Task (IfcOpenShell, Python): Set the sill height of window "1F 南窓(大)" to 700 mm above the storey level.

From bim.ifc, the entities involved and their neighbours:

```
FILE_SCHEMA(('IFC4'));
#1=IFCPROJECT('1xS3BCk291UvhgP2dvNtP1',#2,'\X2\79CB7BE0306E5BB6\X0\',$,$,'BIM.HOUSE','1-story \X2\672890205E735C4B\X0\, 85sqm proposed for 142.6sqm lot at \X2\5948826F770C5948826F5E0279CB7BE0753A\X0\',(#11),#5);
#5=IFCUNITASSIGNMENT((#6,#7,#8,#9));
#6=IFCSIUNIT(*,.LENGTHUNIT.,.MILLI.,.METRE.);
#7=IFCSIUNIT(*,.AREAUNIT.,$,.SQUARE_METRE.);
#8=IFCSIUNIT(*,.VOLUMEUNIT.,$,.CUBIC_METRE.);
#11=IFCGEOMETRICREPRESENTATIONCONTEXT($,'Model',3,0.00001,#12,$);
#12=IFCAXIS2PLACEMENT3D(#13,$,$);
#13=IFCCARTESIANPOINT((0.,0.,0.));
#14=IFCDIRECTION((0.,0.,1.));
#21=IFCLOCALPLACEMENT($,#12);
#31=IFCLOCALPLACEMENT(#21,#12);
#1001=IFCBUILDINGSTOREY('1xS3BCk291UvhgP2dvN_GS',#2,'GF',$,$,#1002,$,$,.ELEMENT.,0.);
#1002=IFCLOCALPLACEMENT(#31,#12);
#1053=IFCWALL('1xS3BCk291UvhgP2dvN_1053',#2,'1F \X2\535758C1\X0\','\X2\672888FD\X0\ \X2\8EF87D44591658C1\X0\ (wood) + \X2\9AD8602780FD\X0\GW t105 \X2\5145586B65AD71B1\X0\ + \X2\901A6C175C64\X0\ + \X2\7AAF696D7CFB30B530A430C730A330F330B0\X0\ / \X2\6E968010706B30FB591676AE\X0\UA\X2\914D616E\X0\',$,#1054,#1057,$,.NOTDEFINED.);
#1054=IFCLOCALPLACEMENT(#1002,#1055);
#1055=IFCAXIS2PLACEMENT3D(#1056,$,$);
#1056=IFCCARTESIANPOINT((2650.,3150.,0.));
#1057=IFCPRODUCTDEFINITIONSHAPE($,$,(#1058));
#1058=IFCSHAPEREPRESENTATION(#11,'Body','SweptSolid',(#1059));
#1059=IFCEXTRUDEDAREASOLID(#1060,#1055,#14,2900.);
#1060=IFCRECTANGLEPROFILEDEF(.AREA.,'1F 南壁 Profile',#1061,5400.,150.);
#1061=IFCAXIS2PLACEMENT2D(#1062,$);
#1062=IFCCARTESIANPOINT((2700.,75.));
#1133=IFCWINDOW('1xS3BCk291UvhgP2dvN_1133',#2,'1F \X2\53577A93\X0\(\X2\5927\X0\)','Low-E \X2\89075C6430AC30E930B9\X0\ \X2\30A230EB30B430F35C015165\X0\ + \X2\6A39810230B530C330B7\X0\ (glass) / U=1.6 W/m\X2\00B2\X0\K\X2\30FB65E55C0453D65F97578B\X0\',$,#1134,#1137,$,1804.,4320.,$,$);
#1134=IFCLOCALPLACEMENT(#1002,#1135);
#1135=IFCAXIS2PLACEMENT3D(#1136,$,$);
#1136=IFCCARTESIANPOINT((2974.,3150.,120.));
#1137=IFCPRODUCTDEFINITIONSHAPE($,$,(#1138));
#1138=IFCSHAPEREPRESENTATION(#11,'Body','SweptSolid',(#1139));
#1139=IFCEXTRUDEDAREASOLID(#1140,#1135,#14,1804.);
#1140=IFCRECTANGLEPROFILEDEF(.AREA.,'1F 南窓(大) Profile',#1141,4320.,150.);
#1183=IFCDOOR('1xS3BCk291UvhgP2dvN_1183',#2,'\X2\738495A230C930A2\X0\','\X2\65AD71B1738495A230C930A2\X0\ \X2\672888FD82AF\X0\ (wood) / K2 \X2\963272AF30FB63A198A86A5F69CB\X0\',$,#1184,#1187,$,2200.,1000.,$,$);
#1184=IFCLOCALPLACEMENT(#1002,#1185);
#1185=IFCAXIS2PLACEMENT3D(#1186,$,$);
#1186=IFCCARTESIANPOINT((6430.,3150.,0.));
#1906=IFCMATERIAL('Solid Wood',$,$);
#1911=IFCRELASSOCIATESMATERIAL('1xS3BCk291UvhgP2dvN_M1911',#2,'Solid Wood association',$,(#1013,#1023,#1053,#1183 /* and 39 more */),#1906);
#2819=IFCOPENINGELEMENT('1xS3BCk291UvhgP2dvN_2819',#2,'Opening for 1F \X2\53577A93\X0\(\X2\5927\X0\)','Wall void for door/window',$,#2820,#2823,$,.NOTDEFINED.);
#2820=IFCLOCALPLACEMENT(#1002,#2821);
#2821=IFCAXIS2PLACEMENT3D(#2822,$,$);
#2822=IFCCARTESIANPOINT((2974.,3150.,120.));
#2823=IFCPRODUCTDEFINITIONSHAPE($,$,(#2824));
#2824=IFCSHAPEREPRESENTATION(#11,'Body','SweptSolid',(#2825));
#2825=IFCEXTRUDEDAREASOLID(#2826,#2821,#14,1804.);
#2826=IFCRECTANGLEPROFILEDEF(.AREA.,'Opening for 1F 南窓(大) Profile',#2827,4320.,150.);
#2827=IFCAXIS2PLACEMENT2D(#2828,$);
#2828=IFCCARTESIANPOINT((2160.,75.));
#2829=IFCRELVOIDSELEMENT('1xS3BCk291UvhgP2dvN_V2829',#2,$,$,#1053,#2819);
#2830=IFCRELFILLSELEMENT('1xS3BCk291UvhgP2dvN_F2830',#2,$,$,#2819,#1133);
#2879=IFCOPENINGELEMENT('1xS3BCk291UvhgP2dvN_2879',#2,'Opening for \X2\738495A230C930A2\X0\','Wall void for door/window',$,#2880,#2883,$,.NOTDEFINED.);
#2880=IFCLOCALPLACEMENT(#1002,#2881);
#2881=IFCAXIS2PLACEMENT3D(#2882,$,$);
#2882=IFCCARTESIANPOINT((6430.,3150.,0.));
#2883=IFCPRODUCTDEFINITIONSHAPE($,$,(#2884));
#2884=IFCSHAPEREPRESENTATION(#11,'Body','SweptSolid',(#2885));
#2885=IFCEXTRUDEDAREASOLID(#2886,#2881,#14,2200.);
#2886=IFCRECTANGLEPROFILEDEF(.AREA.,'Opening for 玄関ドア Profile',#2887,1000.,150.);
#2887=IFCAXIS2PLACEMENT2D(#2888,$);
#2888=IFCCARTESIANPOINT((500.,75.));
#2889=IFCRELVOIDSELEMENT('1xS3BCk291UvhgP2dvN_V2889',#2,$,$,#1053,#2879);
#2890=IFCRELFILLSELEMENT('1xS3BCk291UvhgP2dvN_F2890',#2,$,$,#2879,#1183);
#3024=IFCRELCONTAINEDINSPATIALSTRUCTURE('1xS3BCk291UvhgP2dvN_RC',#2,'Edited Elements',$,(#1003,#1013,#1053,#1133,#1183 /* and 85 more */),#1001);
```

```python
import numpy as np
import ifcopenshell
import ifcopenshell.api.geometry
import ifcopenshell.geom
import ifcopenshell.util.element
import ifcopenshell.util.placement
import ifcopenshell.util.shape
import ifcopenshell.util.unit

model = ifcopenshell.open("bim.ifc")
unit_scale = ifcopenshell.util.unit.calculate_unit_scale(model)

window = model.by_guid("1xS3BCk291UvhgP2dvN_1133")
opening = window.FillsVoids[0].RelatingOpeningElement
storey = ifcopenshell.util.element.get_container(window, ifc_class="IfcBuildingStorey")
level = ifcopenshell.util.placement.get_local_placement(storey.ObjectPlacement)[2, 3]

# The opening's origin need not be at the sill, so measure its lowest point.
shape = ifcopenshell.geom.create_shape(ifcopenshell.geom.settings(), opening)
bottom = ifcopenshell.util.shape.get_shape_bottom_elevation(shape, shape.geometry) / unit_scale
dz = level + 0.7 / unit_scale - bottom

shift = np.array([0.0, 0.0, dz])
# The window is not placed relative to its opening, so move both.
for product in (opening, window):
    matrix = ifcopenshell.util.placement.get_local_placement(product.ObjectPlacement)
    matrix[:3, 3] += shift
    ifcopenshell.api.geometry.edit_object_placement(model, product=product, matrix=matrix, is_si=False)

print(f"moved by {dz * unit_scale:+.3f} m")

model.write("bim_edited.ifc")
```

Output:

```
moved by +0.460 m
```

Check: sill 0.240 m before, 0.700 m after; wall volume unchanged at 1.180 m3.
